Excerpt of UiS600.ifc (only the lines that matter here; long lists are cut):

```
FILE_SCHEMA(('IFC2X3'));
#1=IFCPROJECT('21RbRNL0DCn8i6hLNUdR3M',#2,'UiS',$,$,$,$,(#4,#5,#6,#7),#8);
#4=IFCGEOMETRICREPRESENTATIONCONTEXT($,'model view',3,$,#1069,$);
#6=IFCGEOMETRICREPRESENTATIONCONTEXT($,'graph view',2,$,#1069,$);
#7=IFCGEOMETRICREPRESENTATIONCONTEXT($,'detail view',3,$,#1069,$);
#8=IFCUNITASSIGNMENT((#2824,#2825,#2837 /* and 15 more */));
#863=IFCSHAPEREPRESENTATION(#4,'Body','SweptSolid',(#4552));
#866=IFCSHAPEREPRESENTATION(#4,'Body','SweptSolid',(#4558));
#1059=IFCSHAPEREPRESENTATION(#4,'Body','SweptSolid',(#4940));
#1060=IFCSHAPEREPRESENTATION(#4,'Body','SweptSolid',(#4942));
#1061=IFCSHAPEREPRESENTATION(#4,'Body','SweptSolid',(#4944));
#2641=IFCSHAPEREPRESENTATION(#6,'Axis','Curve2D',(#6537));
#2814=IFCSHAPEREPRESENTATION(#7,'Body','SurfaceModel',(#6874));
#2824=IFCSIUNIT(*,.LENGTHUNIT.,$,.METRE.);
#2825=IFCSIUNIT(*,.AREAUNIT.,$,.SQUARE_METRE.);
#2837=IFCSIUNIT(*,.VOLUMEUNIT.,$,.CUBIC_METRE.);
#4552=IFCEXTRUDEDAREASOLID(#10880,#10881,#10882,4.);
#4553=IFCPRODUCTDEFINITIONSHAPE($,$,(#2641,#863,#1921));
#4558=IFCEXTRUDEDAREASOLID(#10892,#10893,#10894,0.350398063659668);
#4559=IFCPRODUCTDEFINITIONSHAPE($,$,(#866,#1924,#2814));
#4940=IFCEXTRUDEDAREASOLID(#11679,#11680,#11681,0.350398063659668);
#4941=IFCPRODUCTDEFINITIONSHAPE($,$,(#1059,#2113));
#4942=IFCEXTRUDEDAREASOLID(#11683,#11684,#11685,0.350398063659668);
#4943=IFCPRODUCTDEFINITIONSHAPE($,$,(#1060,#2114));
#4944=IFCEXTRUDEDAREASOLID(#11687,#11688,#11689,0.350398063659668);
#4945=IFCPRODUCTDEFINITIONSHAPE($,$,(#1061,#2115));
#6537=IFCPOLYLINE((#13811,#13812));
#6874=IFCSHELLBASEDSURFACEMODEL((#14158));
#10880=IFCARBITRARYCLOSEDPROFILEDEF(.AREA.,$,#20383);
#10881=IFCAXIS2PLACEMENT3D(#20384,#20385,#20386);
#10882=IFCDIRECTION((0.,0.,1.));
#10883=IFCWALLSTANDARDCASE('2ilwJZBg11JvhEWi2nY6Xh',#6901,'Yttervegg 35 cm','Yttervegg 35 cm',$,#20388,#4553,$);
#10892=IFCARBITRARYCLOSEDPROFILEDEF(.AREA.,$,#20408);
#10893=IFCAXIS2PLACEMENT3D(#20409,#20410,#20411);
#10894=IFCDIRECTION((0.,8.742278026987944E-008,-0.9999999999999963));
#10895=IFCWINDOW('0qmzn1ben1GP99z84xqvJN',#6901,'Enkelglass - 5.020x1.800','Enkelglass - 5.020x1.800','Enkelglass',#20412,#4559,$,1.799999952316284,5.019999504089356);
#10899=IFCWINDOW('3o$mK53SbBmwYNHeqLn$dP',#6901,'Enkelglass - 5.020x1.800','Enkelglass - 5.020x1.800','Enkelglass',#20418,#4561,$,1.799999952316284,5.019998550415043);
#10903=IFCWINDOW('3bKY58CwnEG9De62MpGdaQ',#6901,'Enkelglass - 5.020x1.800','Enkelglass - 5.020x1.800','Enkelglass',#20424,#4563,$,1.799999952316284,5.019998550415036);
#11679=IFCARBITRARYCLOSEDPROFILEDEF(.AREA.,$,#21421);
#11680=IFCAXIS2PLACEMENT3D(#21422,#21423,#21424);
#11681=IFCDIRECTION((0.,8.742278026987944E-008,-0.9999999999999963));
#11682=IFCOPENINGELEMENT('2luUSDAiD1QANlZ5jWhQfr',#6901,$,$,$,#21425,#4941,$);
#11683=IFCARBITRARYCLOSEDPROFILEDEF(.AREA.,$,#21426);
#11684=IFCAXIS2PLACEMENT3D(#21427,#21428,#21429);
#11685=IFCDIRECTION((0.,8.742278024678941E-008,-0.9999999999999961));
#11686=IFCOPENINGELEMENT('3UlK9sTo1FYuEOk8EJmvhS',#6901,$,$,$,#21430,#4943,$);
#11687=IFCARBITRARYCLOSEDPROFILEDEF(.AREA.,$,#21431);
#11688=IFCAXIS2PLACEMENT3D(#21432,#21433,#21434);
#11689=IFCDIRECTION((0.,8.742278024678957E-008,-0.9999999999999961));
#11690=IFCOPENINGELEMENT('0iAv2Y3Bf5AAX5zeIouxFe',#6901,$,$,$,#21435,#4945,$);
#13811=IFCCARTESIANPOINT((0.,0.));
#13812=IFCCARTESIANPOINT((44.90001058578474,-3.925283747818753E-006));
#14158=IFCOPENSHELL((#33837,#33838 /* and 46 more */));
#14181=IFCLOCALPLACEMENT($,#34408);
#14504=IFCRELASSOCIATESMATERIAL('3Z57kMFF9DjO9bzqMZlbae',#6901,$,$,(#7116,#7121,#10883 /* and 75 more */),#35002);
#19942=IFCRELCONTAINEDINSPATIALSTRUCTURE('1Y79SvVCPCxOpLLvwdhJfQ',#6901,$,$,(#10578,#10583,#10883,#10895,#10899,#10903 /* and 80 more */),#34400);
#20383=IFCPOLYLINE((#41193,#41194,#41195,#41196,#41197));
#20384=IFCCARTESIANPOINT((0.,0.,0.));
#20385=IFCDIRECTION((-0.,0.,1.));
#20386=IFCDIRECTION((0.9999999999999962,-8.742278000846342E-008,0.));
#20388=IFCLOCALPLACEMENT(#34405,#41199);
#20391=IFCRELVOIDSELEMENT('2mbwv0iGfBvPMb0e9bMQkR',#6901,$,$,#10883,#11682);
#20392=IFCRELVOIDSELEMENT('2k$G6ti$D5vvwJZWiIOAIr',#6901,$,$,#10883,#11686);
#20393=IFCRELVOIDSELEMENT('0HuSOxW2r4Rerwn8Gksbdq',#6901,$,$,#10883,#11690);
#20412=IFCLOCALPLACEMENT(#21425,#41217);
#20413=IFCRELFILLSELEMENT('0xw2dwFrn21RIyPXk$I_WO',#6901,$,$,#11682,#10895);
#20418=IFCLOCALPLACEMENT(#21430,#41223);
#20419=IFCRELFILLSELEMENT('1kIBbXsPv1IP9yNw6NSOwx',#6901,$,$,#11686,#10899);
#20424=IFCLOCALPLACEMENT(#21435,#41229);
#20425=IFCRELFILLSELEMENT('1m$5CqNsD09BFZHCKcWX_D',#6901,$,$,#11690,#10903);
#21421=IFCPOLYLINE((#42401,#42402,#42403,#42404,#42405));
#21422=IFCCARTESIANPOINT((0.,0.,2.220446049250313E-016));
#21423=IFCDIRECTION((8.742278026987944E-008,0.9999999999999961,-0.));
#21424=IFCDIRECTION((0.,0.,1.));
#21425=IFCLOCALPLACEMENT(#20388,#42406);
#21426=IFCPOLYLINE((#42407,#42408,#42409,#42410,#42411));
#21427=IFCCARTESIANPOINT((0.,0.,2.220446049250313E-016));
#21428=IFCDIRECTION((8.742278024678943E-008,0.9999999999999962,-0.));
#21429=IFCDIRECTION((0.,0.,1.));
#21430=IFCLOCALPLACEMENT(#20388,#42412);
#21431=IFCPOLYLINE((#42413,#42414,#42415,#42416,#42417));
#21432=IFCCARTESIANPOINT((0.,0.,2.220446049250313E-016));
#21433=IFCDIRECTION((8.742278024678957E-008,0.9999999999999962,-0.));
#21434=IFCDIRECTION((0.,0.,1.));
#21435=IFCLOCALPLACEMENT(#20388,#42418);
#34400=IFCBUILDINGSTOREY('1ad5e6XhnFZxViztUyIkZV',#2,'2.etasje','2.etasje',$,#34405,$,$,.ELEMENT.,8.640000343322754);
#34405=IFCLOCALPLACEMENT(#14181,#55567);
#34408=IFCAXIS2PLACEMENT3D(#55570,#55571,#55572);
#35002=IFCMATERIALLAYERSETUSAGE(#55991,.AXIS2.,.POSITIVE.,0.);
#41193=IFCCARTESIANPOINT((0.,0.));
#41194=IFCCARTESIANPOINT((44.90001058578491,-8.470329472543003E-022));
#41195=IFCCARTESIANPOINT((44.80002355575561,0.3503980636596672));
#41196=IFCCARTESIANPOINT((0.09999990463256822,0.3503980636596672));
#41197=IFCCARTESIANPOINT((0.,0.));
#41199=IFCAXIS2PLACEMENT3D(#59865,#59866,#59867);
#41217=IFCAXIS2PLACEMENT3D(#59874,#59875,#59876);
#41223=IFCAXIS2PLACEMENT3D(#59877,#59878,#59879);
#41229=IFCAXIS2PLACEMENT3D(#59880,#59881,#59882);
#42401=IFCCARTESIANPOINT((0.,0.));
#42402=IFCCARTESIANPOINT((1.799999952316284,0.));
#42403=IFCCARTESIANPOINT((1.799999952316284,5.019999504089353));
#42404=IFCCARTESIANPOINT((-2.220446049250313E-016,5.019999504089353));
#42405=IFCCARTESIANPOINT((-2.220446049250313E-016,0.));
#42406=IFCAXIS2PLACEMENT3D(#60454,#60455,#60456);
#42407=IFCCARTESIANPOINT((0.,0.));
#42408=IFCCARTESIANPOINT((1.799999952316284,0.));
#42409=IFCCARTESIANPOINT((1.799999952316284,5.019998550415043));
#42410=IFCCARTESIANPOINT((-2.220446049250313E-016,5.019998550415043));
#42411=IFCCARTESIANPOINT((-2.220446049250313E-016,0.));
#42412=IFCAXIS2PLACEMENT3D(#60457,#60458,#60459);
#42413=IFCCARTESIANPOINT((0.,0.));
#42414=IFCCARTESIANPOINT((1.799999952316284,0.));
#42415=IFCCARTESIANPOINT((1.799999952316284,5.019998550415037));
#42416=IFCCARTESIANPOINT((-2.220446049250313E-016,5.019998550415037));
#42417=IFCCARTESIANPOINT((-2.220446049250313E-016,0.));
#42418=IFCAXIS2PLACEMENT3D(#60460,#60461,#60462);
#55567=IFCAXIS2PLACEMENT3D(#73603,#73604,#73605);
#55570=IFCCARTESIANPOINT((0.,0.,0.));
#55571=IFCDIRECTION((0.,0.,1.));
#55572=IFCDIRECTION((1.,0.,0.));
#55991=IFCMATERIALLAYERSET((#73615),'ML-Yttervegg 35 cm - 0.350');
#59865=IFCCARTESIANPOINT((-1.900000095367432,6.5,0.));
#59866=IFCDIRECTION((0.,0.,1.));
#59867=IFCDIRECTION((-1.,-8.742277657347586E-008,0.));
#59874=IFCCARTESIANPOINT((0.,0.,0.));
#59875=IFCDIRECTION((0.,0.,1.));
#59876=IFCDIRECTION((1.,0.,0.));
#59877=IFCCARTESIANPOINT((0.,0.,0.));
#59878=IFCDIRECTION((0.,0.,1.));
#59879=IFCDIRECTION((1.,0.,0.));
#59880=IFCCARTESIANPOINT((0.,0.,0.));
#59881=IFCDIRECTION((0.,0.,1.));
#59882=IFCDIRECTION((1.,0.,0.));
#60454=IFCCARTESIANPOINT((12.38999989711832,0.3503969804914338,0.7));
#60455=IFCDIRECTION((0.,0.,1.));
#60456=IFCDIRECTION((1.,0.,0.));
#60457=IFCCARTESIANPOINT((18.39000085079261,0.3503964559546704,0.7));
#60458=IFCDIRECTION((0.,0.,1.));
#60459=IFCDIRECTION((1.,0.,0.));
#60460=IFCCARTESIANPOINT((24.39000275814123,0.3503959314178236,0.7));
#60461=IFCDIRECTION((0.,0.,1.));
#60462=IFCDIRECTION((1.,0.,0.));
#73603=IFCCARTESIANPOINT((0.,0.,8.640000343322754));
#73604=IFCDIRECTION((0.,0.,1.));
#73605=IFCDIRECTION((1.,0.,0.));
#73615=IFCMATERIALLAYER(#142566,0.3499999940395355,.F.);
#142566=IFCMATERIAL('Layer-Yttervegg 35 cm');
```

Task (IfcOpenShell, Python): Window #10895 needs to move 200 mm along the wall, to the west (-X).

```python
import ifcopenshell
import ifcopenshell.api.geometry
import ifcopenshell.util.placement
import ifcopenshell.util.unit

model = ifcopenshell.open("UiS600.ifc")
unit_scale = ifcopenshell.util.unit.calculate_unit_scale(model)

window = model.by_guid("0qmzn1ben1GP99z84xqvJN")
opening = window.FillsVoids[0].RelatingOpeningElement
wall = opening.VoidsElements[0].RelatingBuildingElement

wall_matrix = ifcopenshell.util.placement.get_local_placement(wall.ObjectPlacement)
shift = wall_matrix[:3, 0] * 0.2 / unit_scale
before = ifcopenshell.util.placement.get_local_placement(window.ObjectPlacement)[:3, 3].copy()

# The window is placed relative to its opening, so it follows when the opening moves.
matrix = ifcopenshell.util.placement.get_local_placement(opening.ObjectPlacement)
matrix[:3, 3] += shift
ifcopenshell.api.geometry.edit_object_placement(
    model, product=opening, matrix=matrix, is_si=False, should_transform_children=True
)

after = ifcopenshell.util.placement.get_local_placement(window.ObjectPlacement)[:3, 3]
print("window moved by", (after - before).round(3) + 0.0)

model.write("UiS600-out.ifc")
```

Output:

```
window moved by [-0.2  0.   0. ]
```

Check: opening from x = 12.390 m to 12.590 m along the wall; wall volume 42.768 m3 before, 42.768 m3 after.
